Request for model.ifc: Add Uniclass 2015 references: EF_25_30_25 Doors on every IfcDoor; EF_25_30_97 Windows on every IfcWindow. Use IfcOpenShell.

First a look at what the model holds.

```python
import ifcopenshell

model = ifcopenshell.open("model.ifc")
print(model.schema)
print("classifications:", [c.Name for c in model.by_type("IfcClassification")])
for ifc_class in ("IfcDoor", "IfcRoof", "IfcStair", "IfcWall", "IfcWindow"):
    print(ifc_class, len(model.by_type(ifc_class)))
```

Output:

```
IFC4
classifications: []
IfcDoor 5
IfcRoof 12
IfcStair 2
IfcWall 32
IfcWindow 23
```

```python
import ifcopenshell
import ifcopenshell.api.classification

model = ifcopenshell.open("model.ifc")

system = ifcopenshell.api.classification.add_classification(model, classification="Uniclass 2015")

codes = {
    "IfcDoor": ("EF_25_30_25", "Doors"),
    "IfcWindow": ("EF_25_30_97", "Windows"),
}
for ifc_class, (code, name) in codes.items():
    products = model.by_type(ifc_class)
    ifcopenshell.api.classification.add_reference(
        model, products=products, classification=system, identification=code, name=name
    )
    print(code, len(products))

model.write("model-out.ifc")
```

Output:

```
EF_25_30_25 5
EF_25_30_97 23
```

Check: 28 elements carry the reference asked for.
